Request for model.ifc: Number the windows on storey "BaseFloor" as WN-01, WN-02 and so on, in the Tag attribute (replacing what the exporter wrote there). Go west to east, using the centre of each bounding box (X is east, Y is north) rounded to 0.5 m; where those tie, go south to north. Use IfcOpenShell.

First a look at what the model holds.

```python
import ifcopenshell
import ifcopenshell.util.element
import ifcopenshell.util.placement

model = ifcopenshell.open("model.ifc")
print(model.schema)
storey = next(s for s in model.by_type("IfcBuildingStorey") if s.Name == "BaseFloor")
windows = [e for e in ifcopenshell.util.element.get_decomposition(storey) if e.is_a("IfcWindow")]
for e in sorted(windows, key=lambda e: e.id()):
    origin = ifcopenshell.util.placement.get_local_placement(e.ObjectPlacement)[:3, 3]
    print(e.id(), e.Tag, e.Name, origin.round(2) + 0.0, sep=" | ")
```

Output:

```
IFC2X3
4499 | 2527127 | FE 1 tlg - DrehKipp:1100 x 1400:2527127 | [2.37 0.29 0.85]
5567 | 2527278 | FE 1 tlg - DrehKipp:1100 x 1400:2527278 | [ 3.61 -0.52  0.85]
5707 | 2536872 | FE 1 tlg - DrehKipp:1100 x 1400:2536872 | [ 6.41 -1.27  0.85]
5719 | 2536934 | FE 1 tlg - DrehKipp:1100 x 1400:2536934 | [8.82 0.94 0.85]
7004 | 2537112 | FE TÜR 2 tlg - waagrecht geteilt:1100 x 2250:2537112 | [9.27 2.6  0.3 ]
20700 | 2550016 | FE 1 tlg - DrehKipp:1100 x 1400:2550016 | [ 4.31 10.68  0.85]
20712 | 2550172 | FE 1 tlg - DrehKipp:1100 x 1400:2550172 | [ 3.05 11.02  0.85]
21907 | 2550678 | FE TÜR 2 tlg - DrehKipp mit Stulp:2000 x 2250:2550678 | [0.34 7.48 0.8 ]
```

```python
import ifcopenshell
import ifcopenshell.geom
import ifcopenshell.util.element
import ifcopenshell.util.shape

model = ifcopenshell.open("model.ifc")
settings = ifcopenshell.geom.settings()
settings.set("use-world-coords", True)


def centre(element):
    shape = ifcopenshell.geom.create_shape(settings, element)
    return ifcopenshell.util.shape.get_bbox_centroid(shape.geometry)


storey = next(s for s in model.by_type("IfcBuildingStorey") if s.Name == "BaseFloor")
windows = [e for e in ifcopenshell.util.element.get_decomposition(storey) if e.is_a("IfcWindow")]

# Insertion points can sit at a corner or the storey origin, so sort by the geometry (in metres).
centres = {e: centre(e) for e in windows}
windows.sort(key=lambda e: (round(centres[e][0] / 0.5), centres[e][1]))

for i, e in enumerate(windows, start=1):
    number = f"WN-{i:02d}"
    e.Tag = number
    print(e.id(), number)

model.write("model_edited.ifc")
```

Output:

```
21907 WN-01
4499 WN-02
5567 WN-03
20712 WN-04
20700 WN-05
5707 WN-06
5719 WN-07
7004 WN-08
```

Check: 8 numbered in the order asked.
